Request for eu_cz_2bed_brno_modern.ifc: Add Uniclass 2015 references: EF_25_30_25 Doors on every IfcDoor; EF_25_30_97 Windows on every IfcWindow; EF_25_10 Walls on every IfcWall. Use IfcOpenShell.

First a look at what the model holds.

```python
import ifcopenshell

model = ifcopenshell.open("eu_cz_2bed_brno_modern.ifc")
print(model.schema)
print("classifications:", [c.Name for c in model.by_type("IfcClassification")])
for ifc_class in ("IfcDoor", "IfcRoof", "IfcStair", "IfcWall", "IfcWindow"):
    print(ifc_class, len(model.by_type(ifc_class)))
```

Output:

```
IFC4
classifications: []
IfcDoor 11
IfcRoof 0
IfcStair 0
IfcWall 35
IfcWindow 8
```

```python
import ifcopenshell
import ifcopenshell.api.classification

model = ifcopenshell.open("eu_cz_2bed_brno_modern.ifc")

system = ifcopenshell.api.classification.add_classification(model, classification="Uniclass 2015")

codes = {
    "IfcDoor": ("EF_25_30_25", "Doors"),
    "IfcWindow": ("EF_25_30_97", "Windows"),
    "IfcWall": ("EF_25_10", "Walls"),
}
for ifc_class, (code, name) in codes.items():
    products = model.by_type(ifc_class)
    ifcopenshell.api.classification.add_reference(
        model, products=products, classification=system, identification=code, name=name
    )
    print(code, len(products))

model.write("eu_cz_2bed_brno_modern-out.ifc")
```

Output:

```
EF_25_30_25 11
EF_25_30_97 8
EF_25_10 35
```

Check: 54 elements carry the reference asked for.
